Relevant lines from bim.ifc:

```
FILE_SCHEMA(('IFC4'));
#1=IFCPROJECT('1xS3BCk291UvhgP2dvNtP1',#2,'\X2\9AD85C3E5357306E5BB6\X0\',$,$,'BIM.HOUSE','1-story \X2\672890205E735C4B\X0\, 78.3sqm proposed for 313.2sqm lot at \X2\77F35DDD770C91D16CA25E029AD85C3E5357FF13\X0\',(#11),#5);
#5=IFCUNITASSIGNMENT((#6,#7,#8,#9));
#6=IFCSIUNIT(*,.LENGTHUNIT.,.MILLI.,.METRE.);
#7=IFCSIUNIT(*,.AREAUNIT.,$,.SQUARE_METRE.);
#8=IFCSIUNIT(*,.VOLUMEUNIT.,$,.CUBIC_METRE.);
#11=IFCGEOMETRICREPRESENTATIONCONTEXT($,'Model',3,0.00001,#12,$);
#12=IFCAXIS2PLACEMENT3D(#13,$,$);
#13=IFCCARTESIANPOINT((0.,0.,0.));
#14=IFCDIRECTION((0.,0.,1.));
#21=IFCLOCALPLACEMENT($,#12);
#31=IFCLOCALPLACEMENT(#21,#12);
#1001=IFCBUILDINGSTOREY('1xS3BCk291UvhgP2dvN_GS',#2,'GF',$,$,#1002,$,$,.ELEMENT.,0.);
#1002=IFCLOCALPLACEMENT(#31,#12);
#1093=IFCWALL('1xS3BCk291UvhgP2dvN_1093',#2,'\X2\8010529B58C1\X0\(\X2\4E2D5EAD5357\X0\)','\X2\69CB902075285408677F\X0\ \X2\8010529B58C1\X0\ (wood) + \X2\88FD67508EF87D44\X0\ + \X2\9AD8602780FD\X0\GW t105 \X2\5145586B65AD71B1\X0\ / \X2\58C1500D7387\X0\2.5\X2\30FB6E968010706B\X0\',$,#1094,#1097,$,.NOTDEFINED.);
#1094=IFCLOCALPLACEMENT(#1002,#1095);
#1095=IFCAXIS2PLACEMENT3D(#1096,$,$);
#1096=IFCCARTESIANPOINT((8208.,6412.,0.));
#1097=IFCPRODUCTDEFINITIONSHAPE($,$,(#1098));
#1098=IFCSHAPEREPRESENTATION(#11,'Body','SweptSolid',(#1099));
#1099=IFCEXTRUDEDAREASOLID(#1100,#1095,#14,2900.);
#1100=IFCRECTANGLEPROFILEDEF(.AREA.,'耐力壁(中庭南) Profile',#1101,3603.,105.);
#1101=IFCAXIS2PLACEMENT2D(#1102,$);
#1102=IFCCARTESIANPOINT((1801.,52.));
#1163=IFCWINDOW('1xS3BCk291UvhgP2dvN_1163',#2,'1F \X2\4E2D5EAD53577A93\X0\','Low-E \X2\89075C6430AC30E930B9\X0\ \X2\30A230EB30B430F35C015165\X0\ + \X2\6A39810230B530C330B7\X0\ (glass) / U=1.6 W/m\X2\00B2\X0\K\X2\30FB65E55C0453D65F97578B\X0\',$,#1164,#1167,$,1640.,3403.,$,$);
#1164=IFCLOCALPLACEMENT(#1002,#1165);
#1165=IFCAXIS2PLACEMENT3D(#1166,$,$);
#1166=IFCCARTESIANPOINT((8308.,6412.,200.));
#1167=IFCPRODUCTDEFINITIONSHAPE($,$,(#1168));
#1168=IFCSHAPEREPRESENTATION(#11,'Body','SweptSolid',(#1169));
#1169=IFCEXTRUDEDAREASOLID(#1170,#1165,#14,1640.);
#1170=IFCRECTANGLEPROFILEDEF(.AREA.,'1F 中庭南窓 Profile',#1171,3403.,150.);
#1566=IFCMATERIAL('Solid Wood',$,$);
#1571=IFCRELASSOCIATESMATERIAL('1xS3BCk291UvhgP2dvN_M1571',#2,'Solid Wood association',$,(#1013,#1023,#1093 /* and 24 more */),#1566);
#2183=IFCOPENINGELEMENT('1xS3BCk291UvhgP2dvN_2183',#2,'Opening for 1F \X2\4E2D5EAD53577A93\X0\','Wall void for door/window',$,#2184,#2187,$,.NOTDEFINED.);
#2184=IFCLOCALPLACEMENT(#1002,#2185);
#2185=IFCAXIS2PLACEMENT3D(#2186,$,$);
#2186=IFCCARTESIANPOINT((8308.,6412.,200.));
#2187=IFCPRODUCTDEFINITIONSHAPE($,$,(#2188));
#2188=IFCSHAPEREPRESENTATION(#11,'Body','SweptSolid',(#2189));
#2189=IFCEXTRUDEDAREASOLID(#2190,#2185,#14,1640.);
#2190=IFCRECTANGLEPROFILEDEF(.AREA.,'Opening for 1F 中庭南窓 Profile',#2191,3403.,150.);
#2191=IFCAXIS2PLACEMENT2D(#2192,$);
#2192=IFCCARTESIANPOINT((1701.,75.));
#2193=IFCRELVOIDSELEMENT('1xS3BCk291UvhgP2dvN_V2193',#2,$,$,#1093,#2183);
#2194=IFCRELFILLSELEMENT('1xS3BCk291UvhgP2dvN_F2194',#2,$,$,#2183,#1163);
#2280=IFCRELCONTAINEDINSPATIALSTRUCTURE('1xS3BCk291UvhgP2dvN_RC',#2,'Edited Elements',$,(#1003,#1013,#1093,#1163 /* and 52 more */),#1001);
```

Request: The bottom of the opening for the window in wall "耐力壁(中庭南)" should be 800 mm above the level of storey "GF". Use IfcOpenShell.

```python
import numpy as np
import ifcopenshell
import ifcopenshell.api.geometry
import ifcopenshell.geom
import ifcopenshell.util.element
import ifcopenshell.util.placement
import ifcopenshell.util.shape
import ifcopenshell.util.unit

model = ifcopenshell.open("bim.ifc")
unit_scale = ifcopenshell.util.unit.calculate_unit_scale(model)

window = model.by_guid("1xS3BCk291UvhgP2dvN_1163")
opening = window.FillsVoids[0].RelatingOpeningElement
storey = ifcopenshell.util.element.get_container(window, ifc_class="IfcBuildingStorey")
level = ifcopenshell.util.placement.get_local_placement(storey.ObjectPlacement)[2, 3]

# The opening's origin need not be at the sill, so measure its lowest point.
shape = ifcopenshell.geom.create_shape(ifcopenshell.geom.settings(), opening)
bottom = ifcopenshell.util.shape.get_shape_bottom_elevation(shape, shape.geometry) / unit_scale
dz = level + 0.8 / unit_scale - bottom

shift = np.array([0.0, 0.0, dz])
# The window is not placed relative to its opening, so move both.
for product in (opening, window):
    matrix = ifcopenshell.util.placement.get_local_placement(product.ObjectPlacement)
    matrix[:3, 3] += shift
    ifcopenshell.api.geometry.edit_object_placement(model, product=product, matrix=matrix, is_si=False)

print(f"moved by {dz * unit_scale:+.3f} m")

model.write("bim-out.ifc")
```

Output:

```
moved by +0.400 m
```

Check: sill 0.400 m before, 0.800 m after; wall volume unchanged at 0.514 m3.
